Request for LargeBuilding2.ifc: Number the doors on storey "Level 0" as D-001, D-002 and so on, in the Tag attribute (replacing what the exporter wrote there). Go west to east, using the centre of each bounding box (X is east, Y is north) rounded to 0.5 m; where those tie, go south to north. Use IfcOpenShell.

First a look at what the model holds.

```python
import ifcopenshell
import ifcopenshell.util.element
import ifcopenshell.util.placement

model = ifcopenshell.open("LargeBuilding2.ifc")
print(model.schema)
storey = next(s for s in model.by_type("IfcBuildingStorey") if s.Name == "Level 0")
doors = [e for e in ifcopenshell.util.element.get_decomposition(storey) if e.is_a("IfcDoor")]
for e in sorted(doors, key=lambda e: e.id()):
    origin = ifcopenshell.util.placement.get_local_placement(e.ObjectPlacement)[:3, 3]
    print(e.id(), e.Tag, e.Name, origin.round(2) + 0.0, sep=" | ")
```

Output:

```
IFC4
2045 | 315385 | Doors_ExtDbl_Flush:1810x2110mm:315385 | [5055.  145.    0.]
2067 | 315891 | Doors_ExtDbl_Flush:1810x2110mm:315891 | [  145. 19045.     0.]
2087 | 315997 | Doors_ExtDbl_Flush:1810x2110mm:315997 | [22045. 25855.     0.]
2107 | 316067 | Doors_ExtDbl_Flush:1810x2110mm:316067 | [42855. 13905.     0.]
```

```python
import ifcopenshell
import ifcopenshell.geom
import ifcopenshell.util.element
import ifcopenshell.util.shape

model = ifcopenshell.open("LargeBuilding2.ifc")
settings = ifcopenshell.geom.settings()
settings.set("use-world-coords", True)


def centre(element):
    shape = ifcopenshell.geom.create_shape(settings, element)
    return ifcopenshell.util.shape.get_bbox_centroid(shape.geometry)


storey = next(s for s in model.by_type("IfcBuildingStorey") if s.Name == "Level 0")
doors = [e for e in ifcopenshell.util.element.get_decomposition(storey) if e.is_a("IfcDoor")]

# Insertion points can sit at a corner or the storey origin, so sort by the geometry (in metres).
centres = {e: centre(e) for e in doors}
doors.sort(key=lambda e: (round(centres[e][0] / 0.5), centres[e][1]))

for i, e in enumerate(doors, start=1):
    number = f"D-0{i:02d}"
    e.Tag = number
    print(e.id(), number)

model.write("LargeBuilding2-out.ifc")
```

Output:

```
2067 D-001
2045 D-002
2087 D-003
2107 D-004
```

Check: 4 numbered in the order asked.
